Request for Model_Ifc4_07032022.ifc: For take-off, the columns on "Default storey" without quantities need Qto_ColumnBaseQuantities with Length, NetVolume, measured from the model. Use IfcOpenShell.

First a look at what the model holds.

```python
import ifcopenshell
import ifcopenshell.util.element
import ifcopenshell.util.unit

model = ifcopenshell.open("Model_Ifc4_07032022.ifc")
print(model.schema)
for unit_type in ("LENGTHUNIT", "AREAUNIT", "VOLUMEUNIT"):
    print(unit_type, ifcopenshell.util.unit.calculate_unit_scale(model, unit_type))
storey = next(s for s in model.by_type("IfcBuildingStorey") if s.Name == "Default storey")
columns = [e for e in ifcopenshell.util.element.get_decomposition(storey) if e.is_a("IfcColumn")]
for e in sorted(columns, key=lambda e: e.id()):
    print(e.id(), e.is_a(), e.Name, list(ifcopenshell.util.element.get_psets(e, qtos_only=True)), sep=" | ")
```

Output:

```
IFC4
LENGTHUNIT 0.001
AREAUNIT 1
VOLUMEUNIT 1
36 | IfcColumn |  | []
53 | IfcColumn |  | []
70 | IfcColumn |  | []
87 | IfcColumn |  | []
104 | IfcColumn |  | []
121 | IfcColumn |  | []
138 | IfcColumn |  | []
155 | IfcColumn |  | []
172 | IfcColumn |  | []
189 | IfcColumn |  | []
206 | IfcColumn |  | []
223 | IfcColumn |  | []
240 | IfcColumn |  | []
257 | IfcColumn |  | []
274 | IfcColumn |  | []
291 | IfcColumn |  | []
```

```python
import ifcopenshell
import ifcopenshell.api.pset
import ifcopenshell.geom
import ifcopenshell.util.element
import ifcopenshell.util.shape
import ifcopenshell.util.unit

model = ifcopenshell.open("Model_Ifc4_07032022.ifc")
unit_scale = ifcopenshell.util.unit.calculate_unit_scale(model)
volume_scale = ifcopenshell.util.unit.calculate_unit_scale(model, "VOLUMEUNIT")
settings = ifcopenshell.geom.settings()

storey = next(s for s in model.by_type("IfcBuildingStorey") if s.Name == "Default storey")
columns = [e for e in ifcopenshell.util.element.get_decomposition(storey) if e.is_a("IfcColumn")]

for e in sorted(columns, key=lambda e: e.id()):
    if ifcopenshell.util.element.get_psets(e, qtos_only=True, should_inherit=False):
        continue
    # Geometry comes back in metres, in the element's own axes.
    shape = ifcopenshell.geom.create_shape(settings, e)
    values = {
        "Length": ifcopenshell.util.shape.get_z(shape.geometry) / unit_scale,
        "NetVolume": ifcopenshell.util.shape.get_volume(shape.geometry) / volume_scale,
    }
    qto = ifcopenshell.api.pset.add_qto(model, product=e, name="Qto_ColumnBaseQuantities")
    ifcopenshell.api.pset.edit_qto(model, qto=qto, properties=values)
    print(e.id(), {k: round(v, 3) for k, v in values.items()})

model.write("Model_Ifc4_07032022_edited.ifc")
```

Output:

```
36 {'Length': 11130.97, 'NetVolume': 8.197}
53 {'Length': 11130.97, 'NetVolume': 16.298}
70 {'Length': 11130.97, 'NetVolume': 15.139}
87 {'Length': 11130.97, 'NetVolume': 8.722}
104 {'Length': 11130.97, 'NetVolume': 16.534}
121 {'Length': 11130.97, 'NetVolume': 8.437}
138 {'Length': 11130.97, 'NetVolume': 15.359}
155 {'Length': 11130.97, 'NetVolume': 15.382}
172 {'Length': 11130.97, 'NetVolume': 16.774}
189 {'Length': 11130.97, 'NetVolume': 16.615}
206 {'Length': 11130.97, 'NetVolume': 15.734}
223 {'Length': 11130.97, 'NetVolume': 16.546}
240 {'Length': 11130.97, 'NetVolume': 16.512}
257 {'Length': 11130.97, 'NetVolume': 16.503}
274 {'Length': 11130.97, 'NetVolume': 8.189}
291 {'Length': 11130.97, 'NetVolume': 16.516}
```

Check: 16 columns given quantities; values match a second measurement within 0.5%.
